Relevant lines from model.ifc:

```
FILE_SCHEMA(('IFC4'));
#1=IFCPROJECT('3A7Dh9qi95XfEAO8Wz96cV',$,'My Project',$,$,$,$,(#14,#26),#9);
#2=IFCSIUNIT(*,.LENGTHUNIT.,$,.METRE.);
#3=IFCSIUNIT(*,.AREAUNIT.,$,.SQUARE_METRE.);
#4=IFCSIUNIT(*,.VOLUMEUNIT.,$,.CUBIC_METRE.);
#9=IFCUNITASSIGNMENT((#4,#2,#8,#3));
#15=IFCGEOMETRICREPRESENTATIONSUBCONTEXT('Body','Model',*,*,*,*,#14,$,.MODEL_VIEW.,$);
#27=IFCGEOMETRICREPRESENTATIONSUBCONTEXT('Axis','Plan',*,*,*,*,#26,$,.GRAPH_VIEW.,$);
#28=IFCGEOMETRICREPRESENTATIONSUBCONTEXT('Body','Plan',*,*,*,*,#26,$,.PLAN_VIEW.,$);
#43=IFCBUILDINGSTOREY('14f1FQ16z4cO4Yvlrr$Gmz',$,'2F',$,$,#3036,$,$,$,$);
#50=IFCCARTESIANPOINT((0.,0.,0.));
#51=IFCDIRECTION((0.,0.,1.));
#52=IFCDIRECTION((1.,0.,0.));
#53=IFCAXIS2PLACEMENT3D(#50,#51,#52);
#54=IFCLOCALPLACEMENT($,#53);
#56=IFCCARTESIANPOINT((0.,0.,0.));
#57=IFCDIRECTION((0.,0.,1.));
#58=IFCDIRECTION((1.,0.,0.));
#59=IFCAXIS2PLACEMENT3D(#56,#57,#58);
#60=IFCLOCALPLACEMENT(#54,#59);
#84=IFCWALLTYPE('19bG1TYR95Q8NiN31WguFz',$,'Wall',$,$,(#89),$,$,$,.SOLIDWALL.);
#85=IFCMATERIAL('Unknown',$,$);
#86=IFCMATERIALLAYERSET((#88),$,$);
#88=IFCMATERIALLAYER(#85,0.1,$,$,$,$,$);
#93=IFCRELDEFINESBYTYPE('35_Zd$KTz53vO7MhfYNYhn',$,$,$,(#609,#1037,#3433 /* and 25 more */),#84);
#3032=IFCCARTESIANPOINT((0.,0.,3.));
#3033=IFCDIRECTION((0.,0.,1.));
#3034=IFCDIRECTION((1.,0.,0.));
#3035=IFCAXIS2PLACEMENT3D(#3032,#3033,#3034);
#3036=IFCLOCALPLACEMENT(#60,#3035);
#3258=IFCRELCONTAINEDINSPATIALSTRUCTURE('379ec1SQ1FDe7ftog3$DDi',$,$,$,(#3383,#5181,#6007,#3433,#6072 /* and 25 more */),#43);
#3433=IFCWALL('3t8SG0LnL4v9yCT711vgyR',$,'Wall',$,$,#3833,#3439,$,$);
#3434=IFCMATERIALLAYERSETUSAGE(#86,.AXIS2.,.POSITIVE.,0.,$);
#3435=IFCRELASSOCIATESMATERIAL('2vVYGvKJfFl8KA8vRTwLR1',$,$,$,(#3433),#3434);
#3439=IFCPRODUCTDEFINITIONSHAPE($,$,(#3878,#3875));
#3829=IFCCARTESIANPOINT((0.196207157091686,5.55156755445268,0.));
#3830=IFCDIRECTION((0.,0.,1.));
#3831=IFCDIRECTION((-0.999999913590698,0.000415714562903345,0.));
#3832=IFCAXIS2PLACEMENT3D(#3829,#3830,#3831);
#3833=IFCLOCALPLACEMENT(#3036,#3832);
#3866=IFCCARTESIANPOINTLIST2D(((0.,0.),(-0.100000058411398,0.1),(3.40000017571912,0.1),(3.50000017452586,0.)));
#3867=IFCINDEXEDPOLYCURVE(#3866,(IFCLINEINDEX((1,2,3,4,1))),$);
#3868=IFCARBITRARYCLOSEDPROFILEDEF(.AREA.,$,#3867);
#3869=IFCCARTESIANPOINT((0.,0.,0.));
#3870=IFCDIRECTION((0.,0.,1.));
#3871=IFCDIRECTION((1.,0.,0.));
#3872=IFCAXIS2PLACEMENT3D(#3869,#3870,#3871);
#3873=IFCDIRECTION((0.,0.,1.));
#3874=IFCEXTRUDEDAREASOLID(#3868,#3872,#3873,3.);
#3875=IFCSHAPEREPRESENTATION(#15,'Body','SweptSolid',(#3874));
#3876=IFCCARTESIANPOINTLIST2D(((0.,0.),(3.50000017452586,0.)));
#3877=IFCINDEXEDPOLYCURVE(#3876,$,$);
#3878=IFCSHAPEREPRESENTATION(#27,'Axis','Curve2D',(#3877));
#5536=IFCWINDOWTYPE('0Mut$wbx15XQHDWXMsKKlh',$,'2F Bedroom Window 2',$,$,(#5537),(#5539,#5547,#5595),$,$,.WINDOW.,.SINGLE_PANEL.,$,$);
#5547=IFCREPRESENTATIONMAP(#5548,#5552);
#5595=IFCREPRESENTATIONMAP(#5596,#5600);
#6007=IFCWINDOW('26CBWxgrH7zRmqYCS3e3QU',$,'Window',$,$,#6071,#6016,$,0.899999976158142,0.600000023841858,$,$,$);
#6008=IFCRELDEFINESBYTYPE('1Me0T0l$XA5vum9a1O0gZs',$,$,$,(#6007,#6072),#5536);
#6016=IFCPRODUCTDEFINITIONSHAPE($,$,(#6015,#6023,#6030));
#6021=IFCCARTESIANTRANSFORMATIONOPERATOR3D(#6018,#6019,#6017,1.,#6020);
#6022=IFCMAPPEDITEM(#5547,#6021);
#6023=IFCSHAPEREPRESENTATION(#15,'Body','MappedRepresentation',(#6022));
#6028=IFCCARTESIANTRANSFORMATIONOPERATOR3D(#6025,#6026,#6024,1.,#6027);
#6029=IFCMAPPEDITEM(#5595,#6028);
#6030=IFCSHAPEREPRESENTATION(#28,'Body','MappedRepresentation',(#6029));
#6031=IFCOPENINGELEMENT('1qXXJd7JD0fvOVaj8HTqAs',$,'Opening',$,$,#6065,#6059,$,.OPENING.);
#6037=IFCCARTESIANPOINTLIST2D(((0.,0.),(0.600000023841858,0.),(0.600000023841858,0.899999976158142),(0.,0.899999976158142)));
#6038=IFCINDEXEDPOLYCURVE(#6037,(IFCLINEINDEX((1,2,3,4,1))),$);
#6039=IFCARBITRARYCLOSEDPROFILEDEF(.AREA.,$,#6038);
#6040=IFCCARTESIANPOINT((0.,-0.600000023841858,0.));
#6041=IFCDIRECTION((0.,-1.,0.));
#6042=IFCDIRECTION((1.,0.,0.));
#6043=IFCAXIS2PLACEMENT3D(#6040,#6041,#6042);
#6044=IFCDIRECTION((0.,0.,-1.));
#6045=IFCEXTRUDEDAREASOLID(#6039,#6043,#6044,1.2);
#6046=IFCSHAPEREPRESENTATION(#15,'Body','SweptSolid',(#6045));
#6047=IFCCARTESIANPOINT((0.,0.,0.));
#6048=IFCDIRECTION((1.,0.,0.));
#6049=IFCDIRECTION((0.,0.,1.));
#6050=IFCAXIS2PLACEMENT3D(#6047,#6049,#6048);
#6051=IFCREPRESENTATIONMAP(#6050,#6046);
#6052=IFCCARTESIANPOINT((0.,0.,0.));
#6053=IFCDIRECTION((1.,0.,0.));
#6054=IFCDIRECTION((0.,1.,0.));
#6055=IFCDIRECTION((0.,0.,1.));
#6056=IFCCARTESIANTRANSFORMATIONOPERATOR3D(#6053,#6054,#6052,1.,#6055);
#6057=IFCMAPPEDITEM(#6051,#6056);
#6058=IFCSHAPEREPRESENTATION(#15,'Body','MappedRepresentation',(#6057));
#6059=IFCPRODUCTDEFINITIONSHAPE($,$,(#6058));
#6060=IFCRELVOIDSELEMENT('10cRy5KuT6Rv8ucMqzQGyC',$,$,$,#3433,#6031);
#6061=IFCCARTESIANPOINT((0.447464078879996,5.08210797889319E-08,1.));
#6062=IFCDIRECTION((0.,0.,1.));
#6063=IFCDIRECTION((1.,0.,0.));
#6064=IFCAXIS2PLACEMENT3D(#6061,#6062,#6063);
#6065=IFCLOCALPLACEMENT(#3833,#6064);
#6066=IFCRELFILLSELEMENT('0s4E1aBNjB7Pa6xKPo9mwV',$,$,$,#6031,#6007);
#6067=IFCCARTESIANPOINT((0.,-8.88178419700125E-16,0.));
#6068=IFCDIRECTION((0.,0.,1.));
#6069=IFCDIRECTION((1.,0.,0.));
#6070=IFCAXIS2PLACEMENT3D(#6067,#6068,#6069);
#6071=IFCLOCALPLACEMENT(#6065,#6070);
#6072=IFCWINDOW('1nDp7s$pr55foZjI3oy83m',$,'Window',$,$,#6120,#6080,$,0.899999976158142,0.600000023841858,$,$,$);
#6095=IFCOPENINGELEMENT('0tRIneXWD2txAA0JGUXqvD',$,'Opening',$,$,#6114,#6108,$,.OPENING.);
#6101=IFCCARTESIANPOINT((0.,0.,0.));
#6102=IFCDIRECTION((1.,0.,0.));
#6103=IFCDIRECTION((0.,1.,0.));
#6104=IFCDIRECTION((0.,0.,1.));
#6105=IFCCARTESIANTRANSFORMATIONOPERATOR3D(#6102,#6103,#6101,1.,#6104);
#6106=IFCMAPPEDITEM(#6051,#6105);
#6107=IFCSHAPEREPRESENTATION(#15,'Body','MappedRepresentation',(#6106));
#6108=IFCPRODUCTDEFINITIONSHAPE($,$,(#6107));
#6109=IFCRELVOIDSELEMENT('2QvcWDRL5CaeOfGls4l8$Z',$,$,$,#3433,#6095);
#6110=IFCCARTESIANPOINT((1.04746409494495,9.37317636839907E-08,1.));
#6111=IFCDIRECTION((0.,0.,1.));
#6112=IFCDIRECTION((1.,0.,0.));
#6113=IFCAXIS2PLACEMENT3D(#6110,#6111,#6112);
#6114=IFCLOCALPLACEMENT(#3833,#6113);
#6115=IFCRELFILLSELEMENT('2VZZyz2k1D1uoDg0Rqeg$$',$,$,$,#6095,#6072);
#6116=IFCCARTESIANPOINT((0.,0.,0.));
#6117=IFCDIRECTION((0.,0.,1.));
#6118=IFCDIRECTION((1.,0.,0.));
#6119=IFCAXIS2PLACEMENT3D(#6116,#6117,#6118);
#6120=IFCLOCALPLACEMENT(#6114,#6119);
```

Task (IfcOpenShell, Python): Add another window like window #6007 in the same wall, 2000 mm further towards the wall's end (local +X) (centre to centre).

```python
import ifcopenshell
import ifcopenshell.api.feature
import ifcopenshell.api.geometry
import ifcopenshell.api.root
import ifcopenshell.geom
import ifcopenshell.util.element
import ifcopenshell.util.placement
import ifcopenshell.util.shape

model = ifcopenshell.open("model.ifc")
settings = ifcopenshell.geom.settings()


def volume(element):
    """Net volume in cubic metres, openings subtracted."""
    shape = ifcopenshell.geom.create_shape(settings, element)
    return ifcopenshell.util.shape.get_volume(shape.geometry)


window = model.by_guid("26CBWxgrH7zRmqYCS3e3QU")
opening = window.FillsVoids[0].RelatingOpeningElement
wall = opening.VoidsElements[0].RelatingBuildingElement
before = volume(wall)
shift = ifcopenshell.util.placement.get_local_placement(wall.ObjectPlacement)[:3, 0] * 2.0

# copy_class copies the void relationship, type, container and properties, but no geometry.
new_opening = ifcopenshell.api.root.copy_class(model, product=opening)
new_opening.Representation = ifcopenshell.util.element.copy_deep(
    model, opening.Representation, exclude=["IfcGeometricRepresentationContext", "IfcRepresentationMap"]
)
new_window = ifcopenshell.api.root.copy_class(model, product=window)
new_window.Representation = ifcopenshell.util.element.copy_deep(
    model, window.Representation, exclude=["IfcGeometricRepresentationContext", "IfcRepresentationMap"]
)
ifcopenshell.api.feature.add_filling(model, opening=new_opening, element=new_window)

for old, new in ((opening, new_opening), (window, new_window)):
    matrix = ifcopenshell.util.placement.get_local_placement(old.ObjectPlacement)
    matrix[:3, 3] += shift
    ifcopenshell.api.geometry.edit_object_placement(model, product=new, matrix=matrix, is_si=False)

after = volume(wall)

print(f"wall volume {before:.3f} -> {after:.3f} m3")

model.write("model_rev.ifc")
```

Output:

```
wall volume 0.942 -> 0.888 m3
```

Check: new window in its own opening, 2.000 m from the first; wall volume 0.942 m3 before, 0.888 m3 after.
